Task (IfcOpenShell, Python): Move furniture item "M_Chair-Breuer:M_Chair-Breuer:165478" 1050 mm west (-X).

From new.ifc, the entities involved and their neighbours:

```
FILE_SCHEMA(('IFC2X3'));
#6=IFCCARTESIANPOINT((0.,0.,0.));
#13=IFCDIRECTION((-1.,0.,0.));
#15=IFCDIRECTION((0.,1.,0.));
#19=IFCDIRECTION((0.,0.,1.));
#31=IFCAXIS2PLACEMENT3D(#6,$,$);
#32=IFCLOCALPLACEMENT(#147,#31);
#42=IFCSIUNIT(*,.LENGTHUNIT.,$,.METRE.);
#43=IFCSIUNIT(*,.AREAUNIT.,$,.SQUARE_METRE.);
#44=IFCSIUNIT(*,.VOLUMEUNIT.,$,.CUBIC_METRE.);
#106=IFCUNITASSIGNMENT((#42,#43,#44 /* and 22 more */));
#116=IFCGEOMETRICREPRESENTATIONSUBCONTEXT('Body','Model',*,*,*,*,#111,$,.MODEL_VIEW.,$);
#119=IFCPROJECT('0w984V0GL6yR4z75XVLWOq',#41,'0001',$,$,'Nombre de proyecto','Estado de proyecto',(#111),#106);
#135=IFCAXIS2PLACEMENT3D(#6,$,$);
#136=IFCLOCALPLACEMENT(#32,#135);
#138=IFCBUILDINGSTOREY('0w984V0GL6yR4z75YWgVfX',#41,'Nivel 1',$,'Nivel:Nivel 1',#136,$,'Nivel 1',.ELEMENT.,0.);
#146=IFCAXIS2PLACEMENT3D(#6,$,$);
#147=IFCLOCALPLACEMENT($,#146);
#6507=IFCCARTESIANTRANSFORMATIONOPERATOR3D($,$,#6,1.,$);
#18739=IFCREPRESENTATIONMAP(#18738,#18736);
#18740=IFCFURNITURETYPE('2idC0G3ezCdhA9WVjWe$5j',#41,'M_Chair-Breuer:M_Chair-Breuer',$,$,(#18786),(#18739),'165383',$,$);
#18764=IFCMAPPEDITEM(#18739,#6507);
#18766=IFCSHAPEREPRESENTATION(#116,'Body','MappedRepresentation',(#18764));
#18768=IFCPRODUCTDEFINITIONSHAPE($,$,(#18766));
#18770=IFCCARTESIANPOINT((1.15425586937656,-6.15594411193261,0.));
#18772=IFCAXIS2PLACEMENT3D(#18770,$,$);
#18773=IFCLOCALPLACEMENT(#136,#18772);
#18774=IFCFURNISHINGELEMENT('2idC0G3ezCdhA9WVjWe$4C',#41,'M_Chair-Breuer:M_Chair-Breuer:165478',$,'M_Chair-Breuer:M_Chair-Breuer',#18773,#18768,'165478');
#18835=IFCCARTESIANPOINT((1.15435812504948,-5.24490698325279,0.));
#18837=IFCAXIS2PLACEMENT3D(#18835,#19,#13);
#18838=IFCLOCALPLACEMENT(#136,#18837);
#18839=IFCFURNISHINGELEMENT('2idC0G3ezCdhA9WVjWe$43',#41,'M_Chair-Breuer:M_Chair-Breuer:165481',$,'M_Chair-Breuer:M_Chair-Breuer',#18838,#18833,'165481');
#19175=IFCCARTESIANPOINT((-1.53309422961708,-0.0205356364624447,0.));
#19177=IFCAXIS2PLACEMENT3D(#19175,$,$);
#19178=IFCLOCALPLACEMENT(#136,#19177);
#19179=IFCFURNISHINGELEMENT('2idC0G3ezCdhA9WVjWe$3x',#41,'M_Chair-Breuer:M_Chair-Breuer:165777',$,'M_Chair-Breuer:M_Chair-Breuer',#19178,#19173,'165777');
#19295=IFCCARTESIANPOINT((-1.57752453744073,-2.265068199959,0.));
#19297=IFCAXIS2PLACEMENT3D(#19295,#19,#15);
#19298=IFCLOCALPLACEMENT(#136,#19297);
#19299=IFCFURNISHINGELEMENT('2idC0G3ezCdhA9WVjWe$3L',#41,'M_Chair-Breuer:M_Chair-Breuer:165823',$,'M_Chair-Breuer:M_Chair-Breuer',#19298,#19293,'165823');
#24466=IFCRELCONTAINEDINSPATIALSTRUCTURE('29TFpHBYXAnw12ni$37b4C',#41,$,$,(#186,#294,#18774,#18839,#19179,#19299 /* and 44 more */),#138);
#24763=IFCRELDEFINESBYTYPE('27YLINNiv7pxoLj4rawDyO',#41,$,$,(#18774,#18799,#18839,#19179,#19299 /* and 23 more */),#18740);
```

```python
import ifcopenshell
import ifcopenshell.api.geometry
import ifcopenshell.util.placement
import ifcopenshell.util.unit

model = ifcopenshell.open("new.ifc")
unit_scale = ifcopenshell.util.unit.calculate_unit_scale(model)

item = model.by_guid("2idC0G3ezCdhA9WVjWe$4C")
matrix = ifcopenshell.util.placement.get_local_placement(item.ObjectPlacement)
matrix[0, 3] -= 1.05 / unit_scale
ifcopenshell.api.geometry.edit_object_placement(model, product=item, matrix=matrix, is_si=False)

print(ifcopenshell.util.placement.get_local_placement(item.ObjectPlacement).round(3) + 0.0)

model.write("new_updated.ifc")
```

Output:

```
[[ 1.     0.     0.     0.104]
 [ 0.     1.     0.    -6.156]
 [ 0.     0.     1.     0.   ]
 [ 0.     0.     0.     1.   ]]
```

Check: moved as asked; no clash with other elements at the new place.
